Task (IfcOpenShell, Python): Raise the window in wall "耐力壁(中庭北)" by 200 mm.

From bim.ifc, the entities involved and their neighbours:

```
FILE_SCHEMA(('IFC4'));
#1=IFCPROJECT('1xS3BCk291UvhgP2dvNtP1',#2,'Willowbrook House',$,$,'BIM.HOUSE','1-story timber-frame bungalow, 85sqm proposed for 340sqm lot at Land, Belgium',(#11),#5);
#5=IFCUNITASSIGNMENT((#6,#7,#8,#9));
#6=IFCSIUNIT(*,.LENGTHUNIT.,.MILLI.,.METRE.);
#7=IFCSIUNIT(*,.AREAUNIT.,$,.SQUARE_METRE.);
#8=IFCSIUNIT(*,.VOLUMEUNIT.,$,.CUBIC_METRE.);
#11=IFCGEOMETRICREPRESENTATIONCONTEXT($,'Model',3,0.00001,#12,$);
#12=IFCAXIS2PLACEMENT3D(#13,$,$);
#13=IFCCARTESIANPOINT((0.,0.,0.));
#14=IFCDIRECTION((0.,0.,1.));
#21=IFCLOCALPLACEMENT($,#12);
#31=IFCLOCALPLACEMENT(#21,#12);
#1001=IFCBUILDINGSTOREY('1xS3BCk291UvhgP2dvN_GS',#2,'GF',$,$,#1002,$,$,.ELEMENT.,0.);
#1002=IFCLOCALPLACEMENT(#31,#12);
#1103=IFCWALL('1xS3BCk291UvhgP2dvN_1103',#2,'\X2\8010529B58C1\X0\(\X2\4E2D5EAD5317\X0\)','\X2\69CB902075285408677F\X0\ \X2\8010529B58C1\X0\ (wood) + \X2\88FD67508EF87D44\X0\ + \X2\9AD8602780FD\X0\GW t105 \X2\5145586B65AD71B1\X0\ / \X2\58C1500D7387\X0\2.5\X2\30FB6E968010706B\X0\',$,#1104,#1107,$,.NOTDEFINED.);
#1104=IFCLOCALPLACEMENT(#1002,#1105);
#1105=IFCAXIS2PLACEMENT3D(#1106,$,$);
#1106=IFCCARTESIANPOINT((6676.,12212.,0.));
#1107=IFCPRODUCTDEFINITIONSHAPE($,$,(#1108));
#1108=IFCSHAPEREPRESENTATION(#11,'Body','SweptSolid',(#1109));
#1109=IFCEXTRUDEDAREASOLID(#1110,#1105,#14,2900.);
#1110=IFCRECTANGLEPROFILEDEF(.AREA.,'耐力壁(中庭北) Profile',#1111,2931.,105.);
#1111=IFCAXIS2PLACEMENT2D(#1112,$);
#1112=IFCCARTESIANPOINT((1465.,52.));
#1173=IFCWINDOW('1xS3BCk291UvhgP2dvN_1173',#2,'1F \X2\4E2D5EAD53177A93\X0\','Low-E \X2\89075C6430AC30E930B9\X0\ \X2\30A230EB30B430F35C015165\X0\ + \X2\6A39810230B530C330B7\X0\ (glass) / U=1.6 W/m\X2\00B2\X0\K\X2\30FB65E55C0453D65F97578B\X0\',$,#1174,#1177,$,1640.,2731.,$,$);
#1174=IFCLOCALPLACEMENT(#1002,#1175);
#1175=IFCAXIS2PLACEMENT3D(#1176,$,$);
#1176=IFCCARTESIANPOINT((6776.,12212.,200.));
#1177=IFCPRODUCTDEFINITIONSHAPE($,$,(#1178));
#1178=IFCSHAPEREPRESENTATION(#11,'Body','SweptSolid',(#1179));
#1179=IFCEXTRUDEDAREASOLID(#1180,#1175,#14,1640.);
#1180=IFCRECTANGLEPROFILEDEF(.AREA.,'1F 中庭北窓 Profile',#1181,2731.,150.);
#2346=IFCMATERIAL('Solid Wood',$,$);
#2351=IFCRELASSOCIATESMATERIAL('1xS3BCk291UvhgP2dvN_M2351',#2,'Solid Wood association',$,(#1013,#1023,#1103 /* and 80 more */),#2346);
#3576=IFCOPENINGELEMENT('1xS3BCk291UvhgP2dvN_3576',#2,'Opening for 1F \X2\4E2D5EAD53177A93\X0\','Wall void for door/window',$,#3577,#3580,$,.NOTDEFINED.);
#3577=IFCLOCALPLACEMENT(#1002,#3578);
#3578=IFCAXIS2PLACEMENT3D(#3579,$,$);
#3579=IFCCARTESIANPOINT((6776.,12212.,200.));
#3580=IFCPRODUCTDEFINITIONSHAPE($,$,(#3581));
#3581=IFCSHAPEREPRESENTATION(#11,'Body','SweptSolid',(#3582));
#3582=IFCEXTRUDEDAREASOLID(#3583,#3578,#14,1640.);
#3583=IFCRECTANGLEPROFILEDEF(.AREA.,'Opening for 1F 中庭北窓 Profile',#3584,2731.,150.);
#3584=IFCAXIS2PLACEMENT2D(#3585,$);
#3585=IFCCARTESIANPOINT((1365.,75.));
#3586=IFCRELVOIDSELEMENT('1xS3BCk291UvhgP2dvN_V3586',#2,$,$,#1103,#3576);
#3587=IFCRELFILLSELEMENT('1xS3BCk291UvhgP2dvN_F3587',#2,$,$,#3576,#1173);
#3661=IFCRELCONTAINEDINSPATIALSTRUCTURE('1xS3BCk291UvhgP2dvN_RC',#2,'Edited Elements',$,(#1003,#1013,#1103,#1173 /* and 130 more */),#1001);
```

```python
import numpy as np
import ifcopenshell
import ifcopenshell.api.geometry
import ifcopenshell.util.placement
import ifcopenshell.util.unit

model = ifcopenshell.open("bim.ifc")
unit_scale = ifcopenshell.util.unit.calculate_unit_scale(model)

window = model.by_id(1173)
opening = window.FillsVoids[0].RelatingOpeningElement
dz = 200.0

shift = np.array([0.0, 0.0, dz])
# The window is not placed relative to its opening, so move both.
for product in (opening, window):
    matrix = ifcopenshell.util.placement.get_local_placement(product.ObjectPlacement)
    matrix[:3, 3] += shift
    ifcopenshell.api.geometry.edit_object_placement(model, product=product, matrix=matrix, is_si=False)

print(f"moved by {dz * unit_scale:+.3f} m")

model.write("bim_rev.ifc")
```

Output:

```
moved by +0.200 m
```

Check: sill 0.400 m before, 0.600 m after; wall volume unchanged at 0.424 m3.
